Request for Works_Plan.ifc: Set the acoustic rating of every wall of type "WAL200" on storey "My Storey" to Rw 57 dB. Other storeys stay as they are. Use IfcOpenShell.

First a look at what the model holds.

```python
import ifcopenshell
import ifcopenshell.util.element

model = ifcopenshell.open("Works_Plan.ifc")
print(model.schema)
storey = next(s for s in model.by_type("IfcBuildingStorey") if s.Name == "My Storey")
walls = [e for e in ifcopenshell.util.element.get_decomposition(storey) if e.is_a("IfcWall")]
seen = {}
for e in walls:
    element_type = ifcopenshell.util.element.get_type(e)
    key = (element_type.Name if element_type != e and element_type else None, ifcopenshell.util.element.get_pset(e, "Pset_WallCommon", "AcousticRating"))
    seen[key] = seen.get(key, 0) + 1
for (name, value), count in sorted(seen.items(), key=str):
    print(count, "x", name, "|", value)
```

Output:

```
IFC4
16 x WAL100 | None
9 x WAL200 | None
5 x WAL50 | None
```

```python
import ifcopenshell
import ifcopenshell.api.pset
import ifcopenshell.util.element

model = ifcopenshell.open("Works_Plan.ifc")

storey = next(s for s in model.by_type("IfcBuildingStorey") if s.Name == "My Storey")
walls = [e for e in ifcopenshell.util.element.get_decomposition(storey) if e.is_a("IfcWall")]

count = 0
for e in walls:
    element_type = ifcopenshell.util.element.get_type(e)
    if element_type in (None, e) or element_type.Name != "WAL200":
        continue
    # add_pset returns the element's existing set when there is one.
    pset = ifcopenshell.api.pset.add_pset(model, product=e, name="Pset_WallCommon")
    ifcopenshell.api.pset.edit_pset(model, pset=pset, properties={"AcousticRating": "Rw 57 dB"})
    count += 1

print(count, "walls updated")

model.write("Works_Plan_rev.ifc")
```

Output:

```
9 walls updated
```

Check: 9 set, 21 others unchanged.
